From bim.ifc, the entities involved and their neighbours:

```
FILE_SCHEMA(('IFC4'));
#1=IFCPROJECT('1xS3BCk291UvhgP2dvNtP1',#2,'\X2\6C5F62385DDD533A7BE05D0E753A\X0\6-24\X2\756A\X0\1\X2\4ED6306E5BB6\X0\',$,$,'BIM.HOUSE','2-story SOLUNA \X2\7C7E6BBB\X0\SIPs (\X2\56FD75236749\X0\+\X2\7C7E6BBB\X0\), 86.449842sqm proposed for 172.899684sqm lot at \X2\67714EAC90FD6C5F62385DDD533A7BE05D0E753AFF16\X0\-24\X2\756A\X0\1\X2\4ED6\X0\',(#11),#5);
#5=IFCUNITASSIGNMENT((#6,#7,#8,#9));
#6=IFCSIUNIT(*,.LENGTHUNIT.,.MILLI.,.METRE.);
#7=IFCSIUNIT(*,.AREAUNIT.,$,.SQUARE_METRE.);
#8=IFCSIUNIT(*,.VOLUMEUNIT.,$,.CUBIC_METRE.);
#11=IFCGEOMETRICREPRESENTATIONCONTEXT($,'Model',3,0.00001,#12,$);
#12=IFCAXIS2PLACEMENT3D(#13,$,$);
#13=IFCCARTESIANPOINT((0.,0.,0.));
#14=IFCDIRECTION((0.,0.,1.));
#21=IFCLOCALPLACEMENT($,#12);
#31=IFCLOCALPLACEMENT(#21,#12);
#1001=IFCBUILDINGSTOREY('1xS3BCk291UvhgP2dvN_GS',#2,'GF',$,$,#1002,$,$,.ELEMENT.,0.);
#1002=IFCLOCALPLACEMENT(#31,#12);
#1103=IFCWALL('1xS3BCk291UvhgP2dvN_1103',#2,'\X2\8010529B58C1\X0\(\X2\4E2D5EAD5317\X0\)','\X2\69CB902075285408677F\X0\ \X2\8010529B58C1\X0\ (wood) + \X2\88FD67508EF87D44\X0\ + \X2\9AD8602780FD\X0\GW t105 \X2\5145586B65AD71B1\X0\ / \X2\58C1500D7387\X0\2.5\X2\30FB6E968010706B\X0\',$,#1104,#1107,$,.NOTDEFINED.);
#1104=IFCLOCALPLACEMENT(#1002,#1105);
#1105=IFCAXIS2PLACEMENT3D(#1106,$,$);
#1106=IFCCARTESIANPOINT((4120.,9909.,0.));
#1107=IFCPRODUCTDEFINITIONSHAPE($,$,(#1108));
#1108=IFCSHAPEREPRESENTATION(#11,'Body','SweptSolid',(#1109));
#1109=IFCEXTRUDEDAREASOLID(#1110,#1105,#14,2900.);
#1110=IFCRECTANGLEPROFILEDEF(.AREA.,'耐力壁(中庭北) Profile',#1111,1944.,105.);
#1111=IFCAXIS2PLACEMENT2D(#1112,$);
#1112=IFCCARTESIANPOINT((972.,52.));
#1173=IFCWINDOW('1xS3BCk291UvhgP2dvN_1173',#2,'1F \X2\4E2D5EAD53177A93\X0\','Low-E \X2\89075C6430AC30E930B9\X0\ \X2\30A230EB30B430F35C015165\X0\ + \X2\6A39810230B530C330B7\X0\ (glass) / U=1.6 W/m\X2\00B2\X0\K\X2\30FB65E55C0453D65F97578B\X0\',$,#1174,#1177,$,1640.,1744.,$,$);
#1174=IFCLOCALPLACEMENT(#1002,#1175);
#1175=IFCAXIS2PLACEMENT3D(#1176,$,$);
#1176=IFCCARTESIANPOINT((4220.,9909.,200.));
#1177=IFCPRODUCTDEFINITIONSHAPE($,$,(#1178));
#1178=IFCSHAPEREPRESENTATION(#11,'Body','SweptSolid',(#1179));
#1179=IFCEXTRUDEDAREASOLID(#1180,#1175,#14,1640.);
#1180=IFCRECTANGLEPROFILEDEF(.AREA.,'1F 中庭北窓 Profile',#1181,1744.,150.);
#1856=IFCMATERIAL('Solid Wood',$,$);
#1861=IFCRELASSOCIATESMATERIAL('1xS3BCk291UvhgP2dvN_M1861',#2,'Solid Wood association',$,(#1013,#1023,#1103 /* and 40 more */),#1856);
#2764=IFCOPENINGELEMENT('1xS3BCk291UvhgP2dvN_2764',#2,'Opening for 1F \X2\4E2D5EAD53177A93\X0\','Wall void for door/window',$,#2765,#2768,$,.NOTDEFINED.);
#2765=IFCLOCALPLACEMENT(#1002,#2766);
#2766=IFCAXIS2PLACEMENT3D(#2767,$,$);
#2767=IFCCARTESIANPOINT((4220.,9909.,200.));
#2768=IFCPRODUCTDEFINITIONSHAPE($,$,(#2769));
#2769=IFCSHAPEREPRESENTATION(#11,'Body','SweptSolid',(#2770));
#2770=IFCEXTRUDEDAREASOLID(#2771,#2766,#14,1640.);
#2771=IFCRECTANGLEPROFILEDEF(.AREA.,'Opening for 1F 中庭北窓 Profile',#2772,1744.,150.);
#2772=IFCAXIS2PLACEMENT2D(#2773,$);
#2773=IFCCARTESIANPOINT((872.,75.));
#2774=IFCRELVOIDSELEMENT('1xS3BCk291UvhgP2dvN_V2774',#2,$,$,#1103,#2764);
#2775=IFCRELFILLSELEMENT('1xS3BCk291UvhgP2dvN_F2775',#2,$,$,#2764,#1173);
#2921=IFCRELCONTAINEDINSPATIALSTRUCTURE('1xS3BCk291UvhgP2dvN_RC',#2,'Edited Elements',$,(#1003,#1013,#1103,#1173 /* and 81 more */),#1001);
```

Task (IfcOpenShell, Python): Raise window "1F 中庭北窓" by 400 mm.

```python
import numpy as np
import ifcopenshell
import ifcopenshell.api.geometry
import ifcopenshell.util.placement
import ifcopenshell.util.unit

model = ifcopenshell.open("bim.ifc")
unit_scale = ifcopenshell.util.unit.calculate_unit_scale(model)

window = model.by_guid("1xS3BCk291UvhgP2dvN_1173")
opening = window.FillsVoids[0].RelatingOpeningElement
dz = 400.0

shift = np.array([0.0, 0.0, dz])
# The window is not placed relative to its opening, so move both.
for product in (opening, window):
    matrix = ifcopenshell.util.placement.get_local_placement(product.ObjectPlacement)
    matrix[:3, 3] += shift
    ifcopenshell.api.geometry.edit_object_placement(model, product=product, matrix=matrix, is_si=False)

print(f"moved by {dz * unit_scale:+.3f} m")

model.write("bim_v2.ifc")
```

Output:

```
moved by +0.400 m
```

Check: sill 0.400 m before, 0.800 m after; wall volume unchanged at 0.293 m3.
